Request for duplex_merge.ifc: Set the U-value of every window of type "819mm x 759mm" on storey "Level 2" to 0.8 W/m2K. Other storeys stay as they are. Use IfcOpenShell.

First a look at what the model holds.

```python
import ifcopenshell
import ifcopenshell.util.element

model = ifcopenshell.open("duplex_merge.ifc")
print(model.schema)
storey = next(s for s in model.by_type("IfcBuildingStorey") if s.Name == "Level 2")
windows = [e for e in ifcopenshell.util.element.get_decomposition(storey) if e.is_a("IfcWindow")]
seen = {}
for e in windows:
    element_type = ifcopenshell.util.element.get_type(e)
    key = (element_type.Name if element_type != e and element_type else None, ifcopenshell.util.element.get_pset(e, "Pset_WindowCommon", "ThermalTransmittance"))
    seen[key] = seen.get(key, 0) + 1
for (name, value), count in sorted(seen.items(), key=str):
    print(count, "x", name, "|", value)
```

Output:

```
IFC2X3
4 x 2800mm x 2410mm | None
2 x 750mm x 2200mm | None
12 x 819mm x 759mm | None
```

```python
import ifcopenshell
import ifcopenshell.api.pset
import ifcopenshell.util.element

model = ifcopenshell.open("duplex_merge.ifc")

storey = next(s for s in model.by_type("IfcBuildingStorey") if s.Name == "Level 2")
windows = [e for e in ifcopenshell.util.element.get_decomposition(storey) if e.is_a("IfcWindow")]

count = 0
for e in windows:
    element_type = ifcopenshell.util.element.get_type(e)
    if element_type in (None, e) or element_type.Name != "819mm x 759mm":
        continue
    # add_pset returns the element's existing set when there is one.
    pset = ifcopenshell.api.pset.add_pset(model, product=e, name="Pset_WindowCommon")
    ifcopenshell.api.pset.edit_pset(model, pset=pset, properties={"ThermalTransmittance": 0.8})
    count += 1

print(count, "windows updated")

model.write("duplex_merge-out.ifc")
```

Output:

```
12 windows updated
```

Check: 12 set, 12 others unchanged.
